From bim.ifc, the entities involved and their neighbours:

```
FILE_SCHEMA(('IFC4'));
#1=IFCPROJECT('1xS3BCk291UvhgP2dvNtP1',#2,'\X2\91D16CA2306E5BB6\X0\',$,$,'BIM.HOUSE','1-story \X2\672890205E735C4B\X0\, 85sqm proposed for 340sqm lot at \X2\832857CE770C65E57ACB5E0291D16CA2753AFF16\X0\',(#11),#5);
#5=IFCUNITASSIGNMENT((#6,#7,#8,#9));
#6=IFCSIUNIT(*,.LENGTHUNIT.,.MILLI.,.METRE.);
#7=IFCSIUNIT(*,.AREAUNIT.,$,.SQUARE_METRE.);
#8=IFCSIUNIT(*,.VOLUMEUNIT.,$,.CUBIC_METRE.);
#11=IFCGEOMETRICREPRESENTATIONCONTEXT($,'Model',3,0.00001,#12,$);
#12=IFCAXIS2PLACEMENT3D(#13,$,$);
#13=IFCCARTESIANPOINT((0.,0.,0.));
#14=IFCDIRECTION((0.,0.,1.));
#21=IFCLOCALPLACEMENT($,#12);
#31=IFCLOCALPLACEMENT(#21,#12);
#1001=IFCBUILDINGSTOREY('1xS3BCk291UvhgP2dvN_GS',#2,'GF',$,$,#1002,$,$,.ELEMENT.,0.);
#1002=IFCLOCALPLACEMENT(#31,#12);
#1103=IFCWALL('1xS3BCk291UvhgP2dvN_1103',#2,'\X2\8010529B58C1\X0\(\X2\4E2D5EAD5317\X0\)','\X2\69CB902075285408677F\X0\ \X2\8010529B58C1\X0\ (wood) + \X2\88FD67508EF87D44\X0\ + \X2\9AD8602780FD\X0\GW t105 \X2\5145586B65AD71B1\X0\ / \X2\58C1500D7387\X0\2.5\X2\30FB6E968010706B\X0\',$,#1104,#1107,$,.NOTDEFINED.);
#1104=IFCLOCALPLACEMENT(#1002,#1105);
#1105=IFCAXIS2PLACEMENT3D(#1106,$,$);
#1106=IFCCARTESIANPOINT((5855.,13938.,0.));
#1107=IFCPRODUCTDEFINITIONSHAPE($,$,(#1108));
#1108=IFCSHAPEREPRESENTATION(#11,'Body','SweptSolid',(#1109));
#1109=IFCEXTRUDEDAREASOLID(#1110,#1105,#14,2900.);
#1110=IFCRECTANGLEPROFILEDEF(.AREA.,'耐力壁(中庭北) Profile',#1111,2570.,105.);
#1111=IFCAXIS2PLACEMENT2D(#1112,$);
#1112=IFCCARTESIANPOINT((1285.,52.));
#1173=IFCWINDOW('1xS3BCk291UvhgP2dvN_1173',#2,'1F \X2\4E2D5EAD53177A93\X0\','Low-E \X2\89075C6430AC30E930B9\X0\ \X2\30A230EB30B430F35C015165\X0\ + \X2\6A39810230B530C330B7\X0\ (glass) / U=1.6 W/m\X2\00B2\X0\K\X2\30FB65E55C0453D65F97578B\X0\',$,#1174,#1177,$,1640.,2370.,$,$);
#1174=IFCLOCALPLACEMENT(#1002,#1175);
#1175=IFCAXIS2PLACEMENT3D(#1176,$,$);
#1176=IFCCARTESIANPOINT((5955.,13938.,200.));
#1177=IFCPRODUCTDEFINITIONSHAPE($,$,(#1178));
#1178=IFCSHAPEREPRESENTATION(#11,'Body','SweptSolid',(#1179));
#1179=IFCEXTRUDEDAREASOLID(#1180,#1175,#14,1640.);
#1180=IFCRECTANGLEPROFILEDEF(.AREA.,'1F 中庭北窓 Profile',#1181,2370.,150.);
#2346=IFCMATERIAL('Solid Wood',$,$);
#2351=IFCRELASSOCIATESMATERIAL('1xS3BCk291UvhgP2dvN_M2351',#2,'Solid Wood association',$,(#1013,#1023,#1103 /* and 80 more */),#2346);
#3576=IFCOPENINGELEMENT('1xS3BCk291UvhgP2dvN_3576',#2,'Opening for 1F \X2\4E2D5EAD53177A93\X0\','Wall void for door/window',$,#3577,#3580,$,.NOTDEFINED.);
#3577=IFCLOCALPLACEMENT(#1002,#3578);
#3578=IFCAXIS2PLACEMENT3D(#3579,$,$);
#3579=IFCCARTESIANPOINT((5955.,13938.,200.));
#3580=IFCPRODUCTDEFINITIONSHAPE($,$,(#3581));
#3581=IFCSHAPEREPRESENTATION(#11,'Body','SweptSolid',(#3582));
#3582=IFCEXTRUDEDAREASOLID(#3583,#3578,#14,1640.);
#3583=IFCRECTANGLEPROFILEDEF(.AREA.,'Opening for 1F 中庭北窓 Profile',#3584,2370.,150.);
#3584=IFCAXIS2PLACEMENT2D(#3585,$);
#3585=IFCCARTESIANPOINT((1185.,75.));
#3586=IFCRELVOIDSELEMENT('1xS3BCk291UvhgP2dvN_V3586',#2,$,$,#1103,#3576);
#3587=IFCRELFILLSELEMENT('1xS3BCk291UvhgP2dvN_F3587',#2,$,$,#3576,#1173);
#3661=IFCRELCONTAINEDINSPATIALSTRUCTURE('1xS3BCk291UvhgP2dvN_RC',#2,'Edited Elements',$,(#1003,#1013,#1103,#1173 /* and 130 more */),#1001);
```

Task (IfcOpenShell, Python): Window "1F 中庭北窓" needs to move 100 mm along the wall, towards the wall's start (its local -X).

```python
import ifcopenshell
import ifcopenshell.api.geometry
import ifcopenshell.util.placement
import ifcopenshell.util.unit

model = ifcopenshell.open("bim.ifc")
unit_scale = ifcopenshell.util.unit.calculate_unit_scale(model)

window = model.by_id(1173)
opening = window.FillsVoids[0].RelatingOpeningElement
wall = opening.VoidsElements[0].RelatingBuildingElement

wall_matrix = ifcopenshell.util.placement.get_local_placement(wall.ObjectPlacement)
shift = wall_matrix[:3, 0] * -0.1 / unit_scale
before = ifcopenshell.util.placement.get_local_placement(window.ObjectPlacement)[:3, 3].copy()

# The window is not placed relative to its opening, so move both.
for product in (opening, window):
    matrix = ifcopenshell.util.placement.get_local_placement(product.ObjectPlacement)
    matrix[:3, 3] += shift
    ifcopenshell.api.geometry.edit_object_placement(model, product=product, matrix=matrix, is_si=False)

after = ifcopenshell.util.placement.get_local_placement(window.ObjectPlacement)[:3, 3]
print("window moved by", (after - before).round(3) + 0.0)

model.write("bim_rev.ifc")
```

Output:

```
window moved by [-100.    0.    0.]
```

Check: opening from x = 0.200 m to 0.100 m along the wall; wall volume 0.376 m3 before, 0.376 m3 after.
